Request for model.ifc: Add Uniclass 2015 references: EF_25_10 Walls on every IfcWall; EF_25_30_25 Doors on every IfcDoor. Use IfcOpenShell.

First a look at what the model holds.

```python
import ifcopenshell

model = ifcopenshell.open("model.ifc")
print(model.schema)
print("classifications:", [c.Name for c in model.by_type("IfcClassification")])
for ifc_class in ("IfcDoor", "IfcRoof", "IfcStair", "IfcWall", "IfcWindow"):
    print(ifc_class, len(model.by_type(ifc_class)))
```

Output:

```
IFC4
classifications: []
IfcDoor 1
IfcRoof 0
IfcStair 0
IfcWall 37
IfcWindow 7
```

```python
import ifcopenshell
import ifcopenshell.api.classification

model = ifcopenshell.open("model.ifc")

system = ifcopenshell.api.classification.add_classification(model, classification="Uniclass 2015")

codes = {
    "IfcWall": ("EF_25_10", "Walls"),
    "IfcDoor": ("EF_25_30_25", "Doors"),
}
for ifc_class, (code, name) in codes.items():
    products = model.by_type(ifc_class)
    ifcopenshell.api.classification.add_reference(
        model, products=products, classification=system, identification=code, name=name
    )
    print(code, len(products))

model.write("model_v2.ifc")
```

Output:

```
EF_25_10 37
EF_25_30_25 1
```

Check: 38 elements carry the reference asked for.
